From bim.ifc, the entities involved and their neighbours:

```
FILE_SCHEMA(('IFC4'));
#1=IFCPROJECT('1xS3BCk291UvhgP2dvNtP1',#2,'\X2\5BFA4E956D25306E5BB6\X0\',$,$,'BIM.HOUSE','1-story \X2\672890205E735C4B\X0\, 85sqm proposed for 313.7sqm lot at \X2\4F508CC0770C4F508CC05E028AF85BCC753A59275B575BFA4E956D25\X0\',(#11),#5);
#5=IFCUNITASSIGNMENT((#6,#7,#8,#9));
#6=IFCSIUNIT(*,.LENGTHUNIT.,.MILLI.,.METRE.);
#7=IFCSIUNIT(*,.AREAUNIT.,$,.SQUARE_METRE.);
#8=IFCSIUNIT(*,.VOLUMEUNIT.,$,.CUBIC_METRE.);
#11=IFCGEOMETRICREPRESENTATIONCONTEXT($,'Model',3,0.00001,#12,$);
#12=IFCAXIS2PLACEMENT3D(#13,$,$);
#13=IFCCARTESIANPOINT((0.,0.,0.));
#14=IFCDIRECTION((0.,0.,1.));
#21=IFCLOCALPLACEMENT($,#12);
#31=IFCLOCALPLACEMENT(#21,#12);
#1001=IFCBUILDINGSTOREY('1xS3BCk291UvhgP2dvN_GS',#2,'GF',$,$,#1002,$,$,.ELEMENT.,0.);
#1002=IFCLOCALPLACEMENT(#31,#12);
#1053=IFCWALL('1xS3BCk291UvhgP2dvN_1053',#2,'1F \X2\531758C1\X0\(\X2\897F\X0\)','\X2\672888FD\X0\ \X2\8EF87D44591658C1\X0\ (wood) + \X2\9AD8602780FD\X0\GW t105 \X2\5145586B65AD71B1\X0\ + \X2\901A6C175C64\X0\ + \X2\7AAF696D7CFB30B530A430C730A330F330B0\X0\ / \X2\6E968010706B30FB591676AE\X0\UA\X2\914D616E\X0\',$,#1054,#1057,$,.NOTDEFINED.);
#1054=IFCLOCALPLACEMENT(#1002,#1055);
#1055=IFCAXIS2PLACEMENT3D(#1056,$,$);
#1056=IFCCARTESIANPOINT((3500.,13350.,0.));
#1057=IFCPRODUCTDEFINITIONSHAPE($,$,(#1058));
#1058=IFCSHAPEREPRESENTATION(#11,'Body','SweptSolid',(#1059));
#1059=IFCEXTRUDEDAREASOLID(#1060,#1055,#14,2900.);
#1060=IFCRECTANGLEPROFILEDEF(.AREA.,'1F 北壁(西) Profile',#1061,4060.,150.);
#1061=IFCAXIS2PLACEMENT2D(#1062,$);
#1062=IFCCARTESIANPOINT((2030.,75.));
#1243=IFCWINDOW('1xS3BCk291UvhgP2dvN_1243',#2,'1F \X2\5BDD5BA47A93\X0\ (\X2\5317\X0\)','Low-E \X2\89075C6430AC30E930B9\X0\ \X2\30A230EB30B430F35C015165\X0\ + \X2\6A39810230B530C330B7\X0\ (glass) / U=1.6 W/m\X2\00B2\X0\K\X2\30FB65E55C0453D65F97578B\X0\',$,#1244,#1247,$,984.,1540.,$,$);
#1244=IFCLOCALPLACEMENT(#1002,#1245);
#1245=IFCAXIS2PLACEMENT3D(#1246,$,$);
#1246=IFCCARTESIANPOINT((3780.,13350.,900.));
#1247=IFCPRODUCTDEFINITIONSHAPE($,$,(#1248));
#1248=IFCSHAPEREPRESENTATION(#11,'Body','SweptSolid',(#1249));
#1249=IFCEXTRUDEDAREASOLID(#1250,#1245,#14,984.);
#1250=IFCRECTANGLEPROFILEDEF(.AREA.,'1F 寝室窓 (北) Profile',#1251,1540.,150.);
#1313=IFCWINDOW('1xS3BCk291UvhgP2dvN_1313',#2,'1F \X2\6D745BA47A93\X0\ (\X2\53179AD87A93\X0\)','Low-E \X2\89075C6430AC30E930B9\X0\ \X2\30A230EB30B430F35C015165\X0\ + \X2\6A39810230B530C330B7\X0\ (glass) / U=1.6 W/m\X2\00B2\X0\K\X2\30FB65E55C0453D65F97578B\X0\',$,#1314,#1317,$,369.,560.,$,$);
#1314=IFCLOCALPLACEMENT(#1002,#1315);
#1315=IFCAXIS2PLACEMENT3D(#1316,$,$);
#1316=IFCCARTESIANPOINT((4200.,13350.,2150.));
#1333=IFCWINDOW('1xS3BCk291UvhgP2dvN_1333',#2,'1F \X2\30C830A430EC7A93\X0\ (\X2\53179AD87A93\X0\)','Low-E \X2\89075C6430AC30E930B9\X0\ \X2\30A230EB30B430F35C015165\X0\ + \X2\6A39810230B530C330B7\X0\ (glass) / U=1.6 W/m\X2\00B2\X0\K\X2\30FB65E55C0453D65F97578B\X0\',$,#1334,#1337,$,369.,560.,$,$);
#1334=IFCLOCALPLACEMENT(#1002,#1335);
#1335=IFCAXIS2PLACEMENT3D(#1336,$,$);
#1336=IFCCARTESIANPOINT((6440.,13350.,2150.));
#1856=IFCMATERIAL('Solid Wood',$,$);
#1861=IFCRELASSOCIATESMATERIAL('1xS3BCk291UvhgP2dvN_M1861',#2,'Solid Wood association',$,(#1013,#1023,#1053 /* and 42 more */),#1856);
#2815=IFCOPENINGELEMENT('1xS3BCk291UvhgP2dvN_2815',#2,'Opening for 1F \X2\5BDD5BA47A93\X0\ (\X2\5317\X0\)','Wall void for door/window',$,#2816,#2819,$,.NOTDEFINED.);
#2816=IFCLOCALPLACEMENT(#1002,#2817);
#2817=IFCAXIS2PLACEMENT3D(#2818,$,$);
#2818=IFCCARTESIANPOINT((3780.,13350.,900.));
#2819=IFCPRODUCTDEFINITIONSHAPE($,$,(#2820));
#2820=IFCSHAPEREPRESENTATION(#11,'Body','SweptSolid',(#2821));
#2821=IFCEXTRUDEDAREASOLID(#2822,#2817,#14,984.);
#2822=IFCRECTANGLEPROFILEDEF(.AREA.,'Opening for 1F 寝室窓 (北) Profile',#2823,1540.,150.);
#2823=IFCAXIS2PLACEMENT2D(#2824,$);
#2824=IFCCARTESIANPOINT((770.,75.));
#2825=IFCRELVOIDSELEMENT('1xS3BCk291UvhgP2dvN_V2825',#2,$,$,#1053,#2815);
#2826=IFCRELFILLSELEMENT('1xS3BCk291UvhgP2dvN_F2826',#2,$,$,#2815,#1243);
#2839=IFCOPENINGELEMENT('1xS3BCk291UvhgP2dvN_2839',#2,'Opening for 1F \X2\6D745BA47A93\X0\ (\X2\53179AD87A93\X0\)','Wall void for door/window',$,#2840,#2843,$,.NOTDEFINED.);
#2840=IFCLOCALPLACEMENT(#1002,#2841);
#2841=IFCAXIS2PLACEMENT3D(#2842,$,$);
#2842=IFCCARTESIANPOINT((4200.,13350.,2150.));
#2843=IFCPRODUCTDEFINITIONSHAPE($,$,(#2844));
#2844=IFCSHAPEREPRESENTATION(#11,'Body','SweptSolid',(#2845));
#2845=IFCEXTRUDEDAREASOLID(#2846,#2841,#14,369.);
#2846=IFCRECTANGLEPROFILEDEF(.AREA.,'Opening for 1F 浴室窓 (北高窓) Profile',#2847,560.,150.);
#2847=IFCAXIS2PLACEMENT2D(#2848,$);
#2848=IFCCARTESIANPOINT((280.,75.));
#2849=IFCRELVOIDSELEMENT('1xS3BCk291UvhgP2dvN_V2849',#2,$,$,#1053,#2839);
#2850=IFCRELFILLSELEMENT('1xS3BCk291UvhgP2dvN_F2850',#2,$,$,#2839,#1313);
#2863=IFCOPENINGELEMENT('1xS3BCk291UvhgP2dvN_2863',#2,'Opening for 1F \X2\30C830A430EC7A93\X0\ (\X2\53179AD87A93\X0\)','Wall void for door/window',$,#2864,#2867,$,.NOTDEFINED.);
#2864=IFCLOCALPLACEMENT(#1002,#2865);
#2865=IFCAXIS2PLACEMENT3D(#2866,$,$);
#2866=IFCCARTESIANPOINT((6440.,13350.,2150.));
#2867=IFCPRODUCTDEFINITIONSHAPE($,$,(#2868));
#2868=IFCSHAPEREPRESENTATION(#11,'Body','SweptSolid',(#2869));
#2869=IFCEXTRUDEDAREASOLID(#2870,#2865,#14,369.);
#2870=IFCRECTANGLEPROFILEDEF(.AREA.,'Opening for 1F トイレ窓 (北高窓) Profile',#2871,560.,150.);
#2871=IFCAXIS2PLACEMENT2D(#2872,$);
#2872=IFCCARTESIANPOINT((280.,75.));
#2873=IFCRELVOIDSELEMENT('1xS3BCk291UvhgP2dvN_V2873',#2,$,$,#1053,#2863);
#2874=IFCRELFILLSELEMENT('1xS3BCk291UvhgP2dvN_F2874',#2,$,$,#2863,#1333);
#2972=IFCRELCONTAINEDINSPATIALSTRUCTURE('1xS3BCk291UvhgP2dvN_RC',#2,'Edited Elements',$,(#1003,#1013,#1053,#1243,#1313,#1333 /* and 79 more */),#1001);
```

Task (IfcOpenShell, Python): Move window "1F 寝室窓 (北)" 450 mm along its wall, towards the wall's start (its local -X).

```python
import ifcopenshell
import ifcopenshell.api.geometry
import ifcopenshell.util.placement
import ifcopenshell.util.unit

model = ifcopenshell.open("bim.ifc")
unit_scale = ifcopenshell.util.unit.calculate_unit_scale(model)

window = model.by_guid("1xS3BCk291UvhgP2dvN_1243")
opening = window.FillsVoids[0].RelatingOpeningElement
wall = opening.VoidsElements[0].RelatingBuildingElement

wall_matrix = ifcopenshell.util.placement.get_local_placement(wall.ObjectPlacement)
shift = wall_matrix[:3, 0] * -0.45 / unit_scale
before = ifcopenshell.util.placement.get_local_placement(window.ObjectPlacement)[:3, 3].copy()

# The window is not placed relative to its opening, so move both.
for product in (opening, window):
    matrix = ifcopenshell.util.placement.get_local_placement(product.ObjectPlacement)
    matrix[:3, 3] += shift
    ifcopenshell.api.geometry.edit_object_placement(model, product=product, matrix=matrix, is_si=False)

after = ifcopenshell.util.placement.get_local_placement(window.ObjectPlacement)[:3, 3]
print("window moved by", (after - before).round(3) + 0.0)

model.write("bim_updated.ifc")
```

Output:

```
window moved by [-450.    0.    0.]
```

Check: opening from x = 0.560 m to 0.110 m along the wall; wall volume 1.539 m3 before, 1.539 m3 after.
